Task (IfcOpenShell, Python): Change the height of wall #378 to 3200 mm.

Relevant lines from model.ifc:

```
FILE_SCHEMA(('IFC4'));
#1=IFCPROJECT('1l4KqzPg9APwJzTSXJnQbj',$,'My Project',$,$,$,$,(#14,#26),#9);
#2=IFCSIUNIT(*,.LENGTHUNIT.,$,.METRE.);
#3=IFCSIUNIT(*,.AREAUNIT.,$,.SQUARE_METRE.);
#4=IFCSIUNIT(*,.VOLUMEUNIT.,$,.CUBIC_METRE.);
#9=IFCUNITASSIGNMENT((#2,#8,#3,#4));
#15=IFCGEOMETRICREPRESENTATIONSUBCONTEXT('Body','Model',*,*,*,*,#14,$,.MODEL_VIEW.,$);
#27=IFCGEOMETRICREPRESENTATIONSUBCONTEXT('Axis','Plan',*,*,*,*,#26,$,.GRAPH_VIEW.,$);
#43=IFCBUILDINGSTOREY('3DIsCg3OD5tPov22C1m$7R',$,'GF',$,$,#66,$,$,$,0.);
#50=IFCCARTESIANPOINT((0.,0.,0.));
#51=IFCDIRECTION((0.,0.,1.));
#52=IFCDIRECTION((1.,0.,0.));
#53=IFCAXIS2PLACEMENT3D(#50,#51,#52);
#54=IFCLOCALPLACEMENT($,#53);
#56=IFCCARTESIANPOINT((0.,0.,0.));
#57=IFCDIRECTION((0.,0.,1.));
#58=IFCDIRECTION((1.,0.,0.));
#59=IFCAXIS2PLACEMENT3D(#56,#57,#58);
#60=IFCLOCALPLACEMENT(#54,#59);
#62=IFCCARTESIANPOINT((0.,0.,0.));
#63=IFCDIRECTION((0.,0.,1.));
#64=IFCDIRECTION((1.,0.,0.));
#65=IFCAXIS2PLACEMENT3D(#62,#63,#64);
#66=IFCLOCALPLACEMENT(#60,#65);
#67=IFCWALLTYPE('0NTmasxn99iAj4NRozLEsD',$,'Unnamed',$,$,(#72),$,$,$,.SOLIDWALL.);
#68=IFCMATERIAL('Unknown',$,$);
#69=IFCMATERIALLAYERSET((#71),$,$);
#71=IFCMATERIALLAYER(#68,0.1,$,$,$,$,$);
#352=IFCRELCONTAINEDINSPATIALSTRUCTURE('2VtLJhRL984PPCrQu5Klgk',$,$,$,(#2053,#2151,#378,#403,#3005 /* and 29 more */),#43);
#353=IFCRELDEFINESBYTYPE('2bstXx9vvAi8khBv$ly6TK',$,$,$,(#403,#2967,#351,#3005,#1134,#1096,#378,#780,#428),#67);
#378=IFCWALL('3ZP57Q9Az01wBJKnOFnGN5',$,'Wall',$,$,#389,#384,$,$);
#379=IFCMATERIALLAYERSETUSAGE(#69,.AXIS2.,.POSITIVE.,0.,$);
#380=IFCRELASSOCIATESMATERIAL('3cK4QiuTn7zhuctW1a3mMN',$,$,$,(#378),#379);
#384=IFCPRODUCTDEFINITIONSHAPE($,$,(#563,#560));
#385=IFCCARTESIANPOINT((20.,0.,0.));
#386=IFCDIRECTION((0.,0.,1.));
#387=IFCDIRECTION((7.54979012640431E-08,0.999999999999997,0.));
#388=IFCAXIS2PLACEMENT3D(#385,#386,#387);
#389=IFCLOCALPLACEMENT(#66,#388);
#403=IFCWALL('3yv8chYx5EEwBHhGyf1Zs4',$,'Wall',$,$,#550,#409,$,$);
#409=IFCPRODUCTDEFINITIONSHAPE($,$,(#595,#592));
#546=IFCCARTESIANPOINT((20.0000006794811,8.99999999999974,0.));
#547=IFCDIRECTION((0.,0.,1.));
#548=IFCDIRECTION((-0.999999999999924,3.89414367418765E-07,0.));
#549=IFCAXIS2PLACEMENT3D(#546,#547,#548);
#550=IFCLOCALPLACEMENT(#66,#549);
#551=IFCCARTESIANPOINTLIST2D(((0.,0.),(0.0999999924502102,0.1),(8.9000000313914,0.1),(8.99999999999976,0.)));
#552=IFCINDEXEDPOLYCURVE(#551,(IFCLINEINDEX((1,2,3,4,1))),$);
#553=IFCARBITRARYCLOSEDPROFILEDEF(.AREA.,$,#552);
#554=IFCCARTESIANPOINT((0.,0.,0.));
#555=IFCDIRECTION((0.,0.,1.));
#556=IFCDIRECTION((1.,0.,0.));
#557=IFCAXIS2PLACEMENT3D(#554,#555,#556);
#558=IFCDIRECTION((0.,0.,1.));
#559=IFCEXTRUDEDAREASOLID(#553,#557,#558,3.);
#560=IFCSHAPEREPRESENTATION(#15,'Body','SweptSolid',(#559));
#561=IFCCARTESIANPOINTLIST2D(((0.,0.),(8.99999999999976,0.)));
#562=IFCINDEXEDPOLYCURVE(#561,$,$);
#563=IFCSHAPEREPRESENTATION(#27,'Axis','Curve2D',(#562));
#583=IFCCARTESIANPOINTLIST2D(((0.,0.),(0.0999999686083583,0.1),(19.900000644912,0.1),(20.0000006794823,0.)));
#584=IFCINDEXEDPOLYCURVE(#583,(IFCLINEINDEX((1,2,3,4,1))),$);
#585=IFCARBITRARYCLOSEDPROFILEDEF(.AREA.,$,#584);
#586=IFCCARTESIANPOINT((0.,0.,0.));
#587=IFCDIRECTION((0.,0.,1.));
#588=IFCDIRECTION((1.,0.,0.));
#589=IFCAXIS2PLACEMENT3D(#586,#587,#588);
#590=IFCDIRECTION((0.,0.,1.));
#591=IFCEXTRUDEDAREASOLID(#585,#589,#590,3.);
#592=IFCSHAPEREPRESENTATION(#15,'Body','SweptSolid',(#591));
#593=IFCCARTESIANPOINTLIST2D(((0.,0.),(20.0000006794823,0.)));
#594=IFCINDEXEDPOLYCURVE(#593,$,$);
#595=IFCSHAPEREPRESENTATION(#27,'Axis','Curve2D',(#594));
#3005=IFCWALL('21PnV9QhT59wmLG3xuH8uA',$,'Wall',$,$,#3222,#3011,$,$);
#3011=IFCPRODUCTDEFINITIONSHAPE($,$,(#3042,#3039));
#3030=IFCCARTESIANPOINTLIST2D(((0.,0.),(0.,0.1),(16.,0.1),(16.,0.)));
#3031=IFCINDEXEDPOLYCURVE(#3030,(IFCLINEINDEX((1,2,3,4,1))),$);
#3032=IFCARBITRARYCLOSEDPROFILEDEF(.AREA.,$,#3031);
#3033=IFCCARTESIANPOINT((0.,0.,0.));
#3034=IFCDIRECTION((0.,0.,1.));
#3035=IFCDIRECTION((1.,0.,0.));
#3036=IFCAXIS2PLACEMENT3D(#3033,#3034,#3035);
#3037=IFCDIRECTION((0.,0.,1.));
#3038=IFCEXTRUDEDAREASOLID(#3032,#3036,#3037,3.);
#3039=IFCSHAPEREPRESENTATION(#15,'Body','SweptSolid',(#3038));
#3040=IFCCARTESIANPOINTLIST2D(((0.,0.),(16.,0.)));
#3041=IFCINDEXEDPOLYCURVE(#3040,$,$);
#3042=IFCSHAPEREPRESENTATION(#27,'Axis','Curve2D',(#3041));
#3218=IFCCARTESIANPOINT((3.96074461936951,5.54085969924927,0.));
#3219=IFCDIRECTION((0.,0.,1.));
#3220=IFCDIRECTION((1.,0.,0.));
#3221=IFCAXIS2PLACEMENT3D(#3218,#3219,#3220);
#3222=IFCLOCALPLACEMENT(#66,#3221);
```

```python
import ifcopenshell
import ifcopenshell.geom
import ifcopenshell.util.representation
import ifcopenshell.util.shape
import ifcopenshell.util.unit

model = ifcopenshell.open("model.ifc")
unit_scale = ifcopenshell.util.unit.calculate_unit_scale(model)
settings = ifcopenshell.geom.settings()


def volume(element):
    """Net volume in cubic metres, openings subtracted."""
    shape = ifcopenshell.geom.create_shape(settings, element)
    return ifcopenshell.util.shape.get_volume(shape.geometry)


wall = model.by_id(378)
before = volume(wall)

body = ifcopenshell.util.representation.get_representation(wall, "Model", "Body")
solid = body.Items[0]
old_height = solid.Depth
solid.Depth = 3.2 / unit_scale
after = volume(wall)

print(f"height {old_height:g} -> {solid.Depth:g}, volume {before:.3f} -> {after:.3f} m3")

model.write("model_edited.ifc")
```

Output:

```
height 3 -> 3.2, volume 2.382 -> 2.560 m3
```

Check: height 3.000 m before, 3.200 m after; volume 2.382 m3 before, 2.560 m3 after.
